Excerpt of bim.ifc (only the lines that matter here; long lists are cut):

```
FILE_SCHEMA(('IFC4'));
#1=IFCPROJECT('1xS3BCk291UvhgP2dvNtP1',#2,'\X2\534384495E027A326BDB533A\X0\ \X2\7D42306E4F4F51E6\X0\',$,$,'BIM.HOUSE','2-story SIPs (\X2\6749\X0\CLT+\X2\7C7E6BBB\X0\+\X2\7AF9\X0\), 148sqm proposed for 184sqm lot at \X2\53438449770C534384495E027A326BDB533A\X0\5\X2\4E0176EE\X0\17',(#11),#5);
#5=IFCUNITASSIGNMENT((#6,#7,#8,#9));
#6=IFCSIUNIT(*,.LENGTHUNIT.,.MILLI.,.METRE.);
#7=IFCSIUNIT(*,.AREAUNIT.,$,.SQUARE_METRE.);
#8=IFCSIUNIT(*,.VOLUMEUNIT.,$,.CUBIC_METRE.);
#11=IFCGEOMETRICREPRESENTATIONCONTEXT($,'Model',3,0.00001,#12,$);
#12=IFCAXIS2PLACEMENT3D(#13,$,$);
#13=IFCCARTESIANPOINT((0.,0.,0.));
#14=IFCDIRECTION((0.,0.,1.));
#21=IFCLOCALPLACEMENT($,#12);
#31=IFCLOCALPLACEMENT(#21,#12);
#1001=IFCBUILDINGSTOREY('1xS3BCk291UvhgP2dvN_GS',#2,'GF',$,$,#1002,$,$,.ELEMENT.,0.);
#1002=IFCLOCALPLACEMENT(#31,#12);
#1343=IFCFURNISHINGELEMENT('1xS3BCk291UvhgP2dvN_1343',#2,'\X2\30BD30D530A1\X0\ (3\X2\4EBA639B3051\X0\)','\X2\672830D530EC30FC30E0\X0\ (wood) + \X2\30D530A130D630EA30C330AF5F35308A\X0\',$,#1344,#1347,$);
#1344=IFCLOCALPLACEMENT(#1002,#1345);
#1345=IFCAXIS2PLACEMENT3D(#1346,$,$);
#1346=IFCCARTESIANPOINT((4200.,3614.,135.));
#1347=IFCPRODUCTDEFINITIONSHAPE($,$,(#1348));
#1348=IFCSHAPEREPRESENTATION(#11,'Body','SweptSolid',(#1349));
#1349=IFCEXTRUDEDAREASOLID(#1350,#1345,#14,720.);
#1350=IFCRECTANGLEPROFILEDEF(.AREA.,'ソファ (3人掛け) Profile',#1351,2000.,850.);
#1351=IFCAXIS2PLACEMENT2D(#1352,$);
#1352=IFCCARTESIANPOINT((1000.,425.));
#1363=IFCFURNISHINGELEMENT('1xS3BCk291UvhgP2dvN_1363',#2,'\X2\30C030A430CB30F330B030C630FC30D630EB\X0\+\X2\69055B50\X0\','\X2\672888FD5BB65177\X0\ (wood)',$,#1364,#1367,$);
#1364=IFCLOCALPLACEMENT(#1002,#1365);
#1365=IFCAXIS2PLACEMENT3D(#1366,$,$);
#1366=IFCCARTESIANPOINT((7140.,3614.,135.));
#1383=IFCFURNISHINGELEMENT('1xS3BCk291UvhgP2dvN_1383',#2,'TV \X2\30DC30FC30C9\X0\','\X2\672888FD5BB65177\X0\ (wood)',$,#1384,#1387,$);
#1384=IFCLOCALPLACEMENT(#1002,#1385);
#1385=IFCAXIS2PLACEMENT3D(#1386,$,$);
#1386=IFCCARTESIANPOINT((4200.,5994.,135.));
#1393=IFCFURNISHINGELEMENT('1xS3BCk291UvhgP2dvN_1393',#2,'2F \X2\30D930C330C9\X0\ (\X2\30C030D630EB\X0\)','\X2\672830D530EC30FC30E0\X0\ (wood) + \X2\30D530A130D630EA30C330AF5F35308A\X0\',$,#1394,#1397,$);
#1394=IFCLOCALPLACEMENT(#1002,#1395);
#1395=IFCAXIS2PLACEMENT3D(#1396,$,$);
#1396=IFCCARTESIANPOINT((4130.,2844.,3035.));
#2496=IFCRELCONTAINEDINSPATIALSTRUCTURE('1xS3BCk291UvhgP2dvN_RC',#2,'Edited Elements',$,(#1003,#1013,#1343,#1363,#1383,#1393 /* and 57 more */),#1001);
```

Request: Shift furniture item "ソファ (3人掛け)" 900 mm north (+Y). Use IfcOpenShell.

```python
import ifcopenshell
import ifcopenshell.api.geometry
import ifcopenshell.util.placement

model = ifcopenshell.open("bim.ifc")

item = model.by_guid("1xS3BCk291UvhgP2dvN_1343")
matrix = ifcopenshell.util.placement.get_local_placement(item.ObjectPlacement)
matrix[1, 3] += 900.0
ifcopenshell.api.geometry.edit_object_placement(model, product=item, matrix=matrix, is_si=False)

print(ifcopenshell.util.placement.get_local_placement(item.ObjectPlacement).round(3) + 0.0)

model.write("bim_edited.ifc")
```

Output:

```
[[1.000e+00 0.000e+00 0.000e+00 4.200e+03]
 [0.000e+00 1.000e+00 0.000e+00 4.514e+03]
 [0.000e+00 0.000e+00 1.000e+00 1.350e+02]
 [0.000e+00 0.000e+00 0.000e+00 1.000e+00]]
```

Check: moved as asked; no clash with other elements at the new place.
